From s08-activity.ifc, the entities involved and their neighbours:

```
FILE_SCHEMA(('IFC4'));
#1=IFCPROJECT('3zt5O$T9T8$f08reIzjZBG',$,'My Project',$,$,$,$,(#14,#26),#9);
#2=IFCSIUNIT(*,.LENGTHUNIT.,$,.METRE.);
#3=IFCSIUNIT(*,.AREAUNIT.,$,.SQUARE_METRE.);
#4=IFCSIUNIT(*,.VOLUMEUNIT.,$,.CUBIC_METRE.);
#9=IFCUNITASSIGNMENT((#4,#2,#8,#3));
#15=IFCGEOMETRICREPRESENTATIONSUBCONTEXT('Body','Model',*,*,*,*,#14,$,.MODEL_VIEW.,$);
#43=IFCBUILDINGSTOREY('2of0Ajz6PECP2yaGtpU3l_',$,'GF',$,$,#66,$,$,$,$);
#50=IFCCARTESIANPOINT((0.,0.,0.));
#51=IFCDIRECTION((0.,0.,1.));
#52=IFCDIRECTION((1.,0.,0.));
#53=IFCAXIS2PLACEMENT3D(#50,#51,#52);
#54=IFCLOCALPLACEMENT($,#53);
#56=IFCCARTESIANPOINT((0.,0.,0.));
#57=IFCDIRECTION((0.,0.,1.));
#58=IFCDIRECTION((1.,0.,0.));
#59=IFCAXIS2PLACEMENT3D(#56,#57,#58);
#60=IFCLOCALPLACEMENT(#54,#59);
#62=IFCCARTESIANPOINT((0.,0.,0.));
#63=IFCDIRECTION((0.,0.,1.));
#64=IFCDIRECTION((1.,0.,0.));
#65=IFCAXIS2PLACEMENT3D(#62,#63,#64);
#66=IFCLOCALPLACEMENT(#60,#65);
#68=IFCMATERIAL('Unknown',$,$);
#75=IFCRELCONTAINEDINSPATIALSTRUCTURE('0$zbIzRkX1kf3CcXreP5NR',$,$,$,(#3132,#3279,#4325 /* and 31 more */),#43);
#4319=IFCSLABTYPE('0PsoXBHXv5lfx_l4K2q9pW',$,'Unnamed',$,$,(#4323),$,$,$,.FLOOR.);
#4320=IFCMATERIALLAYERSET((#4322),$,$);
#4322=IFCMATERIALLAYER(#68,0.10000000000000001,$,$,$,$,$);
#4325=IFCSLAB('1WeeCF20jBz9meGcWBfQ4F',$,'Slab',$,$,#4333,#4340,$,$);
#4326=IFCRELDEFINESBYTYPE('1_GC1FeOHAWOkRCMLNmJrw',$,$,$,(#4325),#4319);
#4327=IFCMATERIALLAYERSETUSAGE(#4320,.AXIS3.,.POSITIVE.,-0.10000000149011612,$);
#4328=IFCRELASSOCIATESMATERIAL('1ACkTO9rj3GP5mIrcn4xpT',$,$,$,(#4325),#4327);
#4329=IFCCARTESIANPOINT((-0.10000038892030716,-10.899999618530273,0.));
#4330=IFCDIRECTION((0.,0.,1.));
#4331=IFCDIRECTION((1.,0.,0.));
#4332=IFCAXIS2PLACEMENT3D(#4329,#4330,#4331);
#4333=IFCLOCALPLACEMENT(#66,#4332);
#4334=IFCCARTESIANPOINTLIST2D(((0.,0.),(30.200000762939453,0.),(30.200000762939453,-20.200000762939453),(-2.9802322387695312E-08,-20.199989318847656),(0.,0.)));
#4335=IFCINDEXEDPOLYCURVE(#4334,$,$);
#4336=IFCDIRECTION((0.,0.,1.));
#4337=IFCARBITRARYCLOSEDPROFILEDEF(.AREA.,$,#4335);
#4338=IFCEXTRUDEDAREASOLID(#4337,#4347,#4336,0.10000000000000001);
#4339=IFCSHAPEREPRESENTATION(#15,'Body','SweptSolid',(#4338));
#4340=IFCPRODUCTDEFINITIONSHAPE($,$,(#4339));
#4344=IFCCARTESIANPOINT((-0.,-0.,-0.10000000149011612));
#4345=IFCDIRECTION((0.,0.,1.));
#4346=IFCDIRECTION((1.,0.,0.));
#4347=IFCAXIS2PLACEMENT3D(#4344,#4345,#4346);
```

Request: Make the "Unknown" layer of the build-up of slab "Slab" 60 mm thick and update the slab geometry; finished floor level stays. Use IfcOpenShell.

```python
import ifcopenshell
import ifcopenshell.util.element
import ifcopenshell.util.representation
import ifcopenshell.util.unit

model = ifcopenshell.open("s08-activity.ifc")
unit_scale = ifcopenshell.util.unit.calculate_unit_scale(model)

layer_set = model.by_id(4320)
layer = next(l for l in layer_set.MaterialLayers if l.Material and l.Material.Name == "Unknown")
change = 0.06 / unit_scale - layer.LayerThickness
layer.LayerThickness += change

# Geometry does not follow the layer set by itself.
slabs = [e for e in ifcopenshell.util.element.get_elements_by_material(model, layer_set) if e.is_a("IfcSlab")]
for slab in sorted(slabs, key=lambda e: e.id()):
    body = ifcopenshell.util.representation.get_representation(slab, "Model", "Body")
    solid = body.Items[0]
    old_depth = solid.Depth
    solid.Depth += change
    # Extruded upwards: lower the start of the extrusion so the top stays.
    x, y, z = solid.Position.Location.Coordinates
    solid.Position.Location = model.createIfcCartesianPoint((x, y, z - change))
    print(slab.id(), f"{old_depth:g} -> {solid.Depth:g}")

# The layers are counted up from the underside, which has moved.
for usage in {ifcopenshell.util.element.get_material(slab) for slab in slabs}:
    usage.OffsetFromReferenceLine -= change

model.write("s08-activity_rev.ifc")
```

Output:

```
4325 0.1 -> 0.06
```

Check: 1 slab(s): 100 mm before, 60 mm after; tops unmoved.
